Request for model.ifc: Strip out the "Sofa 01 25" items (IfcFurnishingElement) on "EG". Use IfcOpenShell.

First a look at what the model holds.

```python
import ifcopenshell
import ifcopenshell.util.element

model = ifcopenshell.open("model.ifc")
print(model.schema)
storey = next(s for s in model.by_type("IfcBuildingStorey") if s.Name == "EG")
furniture = [e for e in ifcopenshell.util.element.get_decomposition(storey) if e.is_a("IfcFurnishingElement")]
seen = {}
for e in furniture:
    element_type = ifcopenshell.util.element.get_type(e)
    name = element_type.Name if element_type not in (None, e) else None
    seen[name] = seen.get(name, 0) + 1
for name, count in sorted(seen.items(), key=str):
    print(count, "x", name)
```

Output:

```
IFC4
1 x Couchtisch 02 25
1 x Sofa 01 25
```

```python
import ifcopenshell
import ifcopenshell.api.root
import ifcopenshell.util.element

model = ifcopenshell.open("model.ifc")

storey = next(s for s in model.by_type("IfcBuildingStorey") if s.Name == "EG")
furniture = [e for e in ifcopenshell.util.element.get_decomposition(storey) if e.is_a("IfcFurnishingElement")]
targets = [e for e in furniture if (t := ifcopenshell.util.element.get_type(e)) not in (None, e) and t.Name == "Sofa 01 25"]

for e in targets:
    ifcopenshell.api.root.remove_product(model, product=e)
print(len(targets), "removed")

model.write("model-out.ifc")
```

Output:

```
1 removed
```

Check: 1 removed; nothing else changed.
